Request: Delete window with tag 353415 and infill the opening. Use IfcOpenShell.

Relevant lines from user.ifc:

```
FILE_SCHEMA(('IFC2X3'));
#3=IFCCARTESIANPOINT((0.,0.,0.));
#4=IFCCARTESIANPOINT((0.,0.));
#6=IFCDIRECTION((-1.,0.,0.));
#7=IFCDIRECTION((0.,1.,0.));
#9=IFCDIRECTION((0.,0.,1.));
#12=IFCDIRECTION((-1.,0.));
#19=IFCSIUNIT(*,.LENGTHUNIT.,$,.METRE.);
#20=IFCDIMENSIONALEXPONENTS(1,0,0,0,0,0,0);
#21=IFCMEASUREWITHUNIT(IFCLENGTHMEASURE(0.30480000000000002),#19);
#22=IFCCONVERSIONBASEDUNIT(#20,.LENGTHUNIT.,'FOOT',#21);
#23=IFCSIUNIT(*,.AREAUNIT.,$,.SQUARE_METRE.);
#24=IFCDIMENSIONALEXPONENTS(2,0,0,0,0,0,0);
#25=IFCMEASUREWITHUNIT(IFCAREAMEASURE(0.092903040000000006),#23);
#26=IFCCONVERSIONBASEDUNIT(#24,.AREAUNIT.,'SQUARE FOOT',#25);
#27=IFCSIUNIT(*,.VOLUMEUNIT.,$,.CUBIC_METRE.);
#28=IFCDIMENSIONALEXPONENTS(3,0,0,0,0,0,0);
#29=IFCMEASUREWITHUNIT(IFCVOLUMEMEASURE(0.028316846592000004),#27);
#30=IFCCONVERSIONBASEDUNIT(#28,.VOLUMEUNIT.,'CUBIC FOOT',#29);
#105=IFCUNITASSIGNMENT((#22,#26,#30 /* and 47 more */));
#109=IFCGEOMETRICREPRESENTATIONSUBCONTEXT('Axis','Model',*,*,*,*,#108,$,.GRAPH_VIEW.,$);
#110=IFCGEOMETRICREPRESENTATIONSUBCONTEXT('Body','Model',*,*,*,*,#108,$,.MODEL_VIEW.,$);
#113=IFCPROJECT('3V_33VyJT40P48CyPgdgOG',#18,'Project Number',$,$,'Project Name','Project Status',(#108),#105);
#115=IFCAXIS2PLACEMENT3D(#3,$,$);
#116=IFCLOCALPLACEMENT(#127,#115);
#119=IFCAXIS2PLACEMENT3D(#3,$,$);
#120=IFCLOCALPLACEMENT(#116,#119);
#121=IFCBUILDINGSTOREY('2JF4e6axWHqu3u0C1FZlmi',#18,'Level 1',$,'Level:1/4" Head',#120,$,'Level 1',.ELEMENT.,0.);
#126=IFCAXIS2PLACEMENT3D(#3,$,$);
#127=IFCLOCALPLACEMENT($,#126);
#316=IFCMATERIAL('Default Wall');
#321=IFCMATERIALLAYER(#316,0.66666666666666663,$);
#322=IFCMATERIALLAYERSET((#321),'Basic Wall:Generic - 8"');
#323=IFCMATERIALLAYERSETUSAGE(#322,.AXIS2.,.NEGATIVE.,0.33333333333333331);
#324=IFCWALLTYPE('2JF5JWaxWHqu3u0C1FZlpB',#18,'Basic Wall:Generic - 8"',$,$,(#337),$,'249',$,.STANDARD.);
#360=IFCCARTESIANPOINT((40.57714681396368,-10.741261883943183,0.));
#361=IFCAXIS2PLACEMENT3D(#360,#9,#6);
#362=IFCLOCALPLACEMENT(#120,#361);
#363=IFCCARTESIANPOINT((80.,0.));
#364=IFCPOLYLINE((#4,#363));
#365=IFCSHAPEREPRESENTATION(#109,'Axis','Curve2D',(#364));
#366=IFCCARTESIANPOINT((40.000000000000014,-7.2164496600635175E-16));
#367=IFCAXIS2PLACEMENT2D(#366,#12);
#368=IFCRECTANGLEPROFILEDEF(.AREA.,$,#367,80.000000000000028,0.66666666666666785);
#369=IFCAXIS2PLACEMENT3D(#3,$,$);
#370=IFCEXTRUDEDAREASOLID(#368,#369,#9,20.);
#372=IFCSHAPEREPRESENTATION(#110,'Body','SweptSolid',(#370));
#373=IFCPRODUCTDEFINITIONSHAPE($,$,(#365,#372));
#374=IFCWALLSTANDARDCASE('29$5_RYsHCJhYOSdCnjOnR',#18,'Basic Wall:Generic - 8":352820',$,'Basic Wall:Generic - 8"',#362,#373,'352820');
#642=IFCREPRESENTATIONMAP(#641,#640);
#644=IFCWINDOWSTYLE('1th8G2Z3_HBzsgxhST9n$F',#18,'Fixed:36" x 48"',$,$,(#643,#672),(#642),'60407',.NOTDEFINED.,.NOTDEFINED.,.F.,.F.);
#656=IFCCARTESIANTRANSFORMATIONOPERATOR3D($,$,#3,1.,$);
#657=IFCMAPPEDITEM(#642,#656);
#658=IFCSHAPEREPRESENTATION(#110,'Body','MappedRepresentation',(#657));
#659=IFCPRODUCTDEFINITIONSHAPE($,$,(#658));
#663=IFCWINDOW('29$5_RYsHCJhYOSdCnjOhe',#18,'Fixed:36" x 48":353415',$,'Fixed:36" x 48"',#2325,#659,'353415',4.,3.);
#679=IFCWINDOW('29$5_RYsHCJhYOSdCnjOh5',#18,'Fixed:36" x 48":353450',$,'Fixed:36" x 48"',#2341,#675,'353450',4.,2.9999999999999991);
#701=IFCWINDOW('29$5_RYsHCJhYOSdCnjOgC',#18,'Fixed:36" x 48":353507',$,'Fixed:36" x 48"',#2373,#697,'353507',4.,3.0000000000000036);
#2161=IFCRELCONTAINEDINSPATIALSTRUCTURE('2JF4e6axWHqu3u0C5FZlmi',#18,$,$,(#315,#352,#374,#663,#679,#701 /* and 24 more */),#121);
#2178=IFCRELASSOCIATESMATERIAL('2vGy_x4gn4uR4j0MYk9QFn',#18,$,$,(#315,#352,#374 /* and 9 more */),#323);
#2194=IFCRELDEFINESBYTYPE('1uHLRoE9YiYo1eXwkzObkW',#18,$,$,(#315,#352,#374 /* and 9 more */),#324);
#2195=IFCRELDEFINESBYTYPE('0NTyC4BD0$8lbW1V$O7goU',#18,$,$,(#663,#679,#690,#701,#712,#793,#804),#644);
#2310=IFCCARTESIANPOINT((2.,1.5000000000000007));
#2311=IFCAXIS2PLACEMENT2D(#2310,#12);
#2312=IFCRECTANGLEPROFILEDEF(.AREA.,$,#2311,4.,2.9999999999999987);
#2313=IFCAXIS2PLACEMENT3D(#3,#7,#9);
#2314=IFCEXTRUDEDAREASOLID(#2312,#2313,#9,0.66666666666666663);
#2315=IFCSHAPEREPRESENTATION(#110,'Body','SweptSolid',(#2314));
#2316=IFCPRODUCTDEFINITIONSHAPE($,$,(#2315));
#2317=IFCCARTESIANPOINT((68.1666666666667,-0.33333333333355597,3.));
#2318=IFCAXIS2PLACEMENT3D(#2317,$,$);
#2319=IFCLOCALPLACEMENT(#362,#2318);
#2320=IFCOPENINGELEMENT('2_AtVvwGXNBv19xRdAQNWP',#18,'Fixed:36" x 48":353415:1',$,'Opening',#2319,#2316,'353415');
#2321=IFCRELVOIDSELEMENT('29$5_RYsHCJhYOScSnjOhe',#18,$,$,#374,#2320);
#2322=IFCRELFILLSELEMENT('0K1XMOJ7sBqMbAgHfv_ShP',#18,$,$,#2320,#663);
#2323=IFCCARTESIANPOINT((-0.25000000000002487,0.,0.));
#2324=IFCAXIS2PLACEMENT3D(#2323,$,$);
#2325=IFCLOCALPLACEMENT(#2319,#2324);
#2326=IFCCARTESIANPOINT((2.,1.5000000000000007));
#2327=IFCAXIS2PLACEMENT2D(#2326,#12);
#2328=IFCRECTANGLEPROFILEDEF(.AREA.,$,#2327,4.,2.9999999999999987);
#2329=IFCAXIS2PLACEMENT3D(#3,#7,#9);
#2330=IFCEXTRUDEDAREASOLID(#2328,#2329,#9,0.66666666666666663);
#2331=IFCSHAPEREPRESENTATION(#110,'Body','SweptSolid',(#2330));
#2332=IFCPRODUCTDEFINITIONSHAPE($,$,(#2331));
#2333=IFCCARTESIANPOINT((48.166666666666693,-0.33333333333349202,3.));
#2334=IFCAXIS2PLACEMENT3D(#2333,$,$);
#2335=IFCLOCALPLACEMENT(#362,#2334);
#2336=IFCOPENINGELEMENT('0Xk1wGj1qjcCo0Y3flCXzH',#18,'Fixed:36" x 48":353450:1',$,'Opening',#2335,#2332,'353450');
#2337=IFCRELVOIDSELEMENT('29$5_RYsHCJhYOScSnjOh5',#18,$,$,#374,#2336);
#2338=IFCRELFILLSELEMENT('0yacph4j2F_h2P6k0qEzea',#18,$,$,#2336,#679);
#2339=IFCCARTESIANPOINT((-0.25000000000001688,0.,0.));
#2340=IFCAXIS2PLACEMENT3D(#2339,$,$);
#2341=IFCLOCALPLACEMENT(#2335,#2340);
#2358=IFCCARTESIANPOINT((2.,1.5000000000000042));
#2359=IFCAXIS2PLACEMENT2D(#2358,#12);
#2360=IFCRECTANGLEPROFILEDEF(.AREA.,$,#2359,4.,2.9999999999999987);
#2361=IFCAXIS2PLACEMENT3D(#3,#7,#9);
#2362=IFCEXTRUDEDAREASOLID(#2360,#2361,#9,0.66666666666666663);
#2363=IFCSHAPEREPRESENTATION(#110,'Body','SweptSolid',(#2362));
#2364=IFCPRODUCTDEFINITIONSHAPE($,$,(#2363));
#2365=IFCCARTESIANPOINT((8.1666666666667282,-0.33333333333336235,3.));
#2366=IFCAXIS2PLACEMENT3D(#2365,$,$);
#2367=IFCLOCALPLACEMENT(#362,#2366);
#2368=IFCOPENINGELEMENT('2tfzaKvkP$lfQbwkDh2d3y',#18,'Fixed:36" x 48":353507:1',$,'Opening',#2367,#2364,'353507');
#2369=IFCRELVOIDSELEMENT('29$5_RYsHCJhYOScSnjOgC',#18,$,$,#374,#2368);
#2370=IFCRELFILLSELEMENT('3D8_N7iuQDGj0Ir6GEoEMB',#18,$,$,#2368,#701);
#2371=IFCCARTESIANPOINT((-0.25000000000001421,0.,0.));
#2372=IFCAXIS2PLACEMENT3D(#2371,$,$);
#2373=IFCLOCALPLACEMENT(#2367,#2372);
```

```python
import ifcopenshell
import ifcopenshell.api.feature
import ifcopenshell.api.root
import ifcopenshell.geom
import ifcopenshell.util.shape

model = ifcopenshell.open("user.ifc")
settings = ifcopenshell.geom.settings()


def volume(element):
    """Net volume in cubic metres, openings subtracted."""
    shape = ifcopenshell.geom.create_shape(settings, element)
    return ifcopenshell.util.shape.get_volume(shape.geometry)


window = model.by_id(663)
opening = window.FillsVoids[0].RelatingOpeningElement
wall = opening.VoidsElements[0].RelatingBuildingElement
before = volume(wall)

ifcopenshell.api.root.remove_product(model, product=window)
ifcopenshell.api.feature.remove_feature(model, feature=opening)

after = volume(wall)

print(f"wall volume {before:.3f} -> {after:.3f} m3")

model.write("user_v2.ifc")
```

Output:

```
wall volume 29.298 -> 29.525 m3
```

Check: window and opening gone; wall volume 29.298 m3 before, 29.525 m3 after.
